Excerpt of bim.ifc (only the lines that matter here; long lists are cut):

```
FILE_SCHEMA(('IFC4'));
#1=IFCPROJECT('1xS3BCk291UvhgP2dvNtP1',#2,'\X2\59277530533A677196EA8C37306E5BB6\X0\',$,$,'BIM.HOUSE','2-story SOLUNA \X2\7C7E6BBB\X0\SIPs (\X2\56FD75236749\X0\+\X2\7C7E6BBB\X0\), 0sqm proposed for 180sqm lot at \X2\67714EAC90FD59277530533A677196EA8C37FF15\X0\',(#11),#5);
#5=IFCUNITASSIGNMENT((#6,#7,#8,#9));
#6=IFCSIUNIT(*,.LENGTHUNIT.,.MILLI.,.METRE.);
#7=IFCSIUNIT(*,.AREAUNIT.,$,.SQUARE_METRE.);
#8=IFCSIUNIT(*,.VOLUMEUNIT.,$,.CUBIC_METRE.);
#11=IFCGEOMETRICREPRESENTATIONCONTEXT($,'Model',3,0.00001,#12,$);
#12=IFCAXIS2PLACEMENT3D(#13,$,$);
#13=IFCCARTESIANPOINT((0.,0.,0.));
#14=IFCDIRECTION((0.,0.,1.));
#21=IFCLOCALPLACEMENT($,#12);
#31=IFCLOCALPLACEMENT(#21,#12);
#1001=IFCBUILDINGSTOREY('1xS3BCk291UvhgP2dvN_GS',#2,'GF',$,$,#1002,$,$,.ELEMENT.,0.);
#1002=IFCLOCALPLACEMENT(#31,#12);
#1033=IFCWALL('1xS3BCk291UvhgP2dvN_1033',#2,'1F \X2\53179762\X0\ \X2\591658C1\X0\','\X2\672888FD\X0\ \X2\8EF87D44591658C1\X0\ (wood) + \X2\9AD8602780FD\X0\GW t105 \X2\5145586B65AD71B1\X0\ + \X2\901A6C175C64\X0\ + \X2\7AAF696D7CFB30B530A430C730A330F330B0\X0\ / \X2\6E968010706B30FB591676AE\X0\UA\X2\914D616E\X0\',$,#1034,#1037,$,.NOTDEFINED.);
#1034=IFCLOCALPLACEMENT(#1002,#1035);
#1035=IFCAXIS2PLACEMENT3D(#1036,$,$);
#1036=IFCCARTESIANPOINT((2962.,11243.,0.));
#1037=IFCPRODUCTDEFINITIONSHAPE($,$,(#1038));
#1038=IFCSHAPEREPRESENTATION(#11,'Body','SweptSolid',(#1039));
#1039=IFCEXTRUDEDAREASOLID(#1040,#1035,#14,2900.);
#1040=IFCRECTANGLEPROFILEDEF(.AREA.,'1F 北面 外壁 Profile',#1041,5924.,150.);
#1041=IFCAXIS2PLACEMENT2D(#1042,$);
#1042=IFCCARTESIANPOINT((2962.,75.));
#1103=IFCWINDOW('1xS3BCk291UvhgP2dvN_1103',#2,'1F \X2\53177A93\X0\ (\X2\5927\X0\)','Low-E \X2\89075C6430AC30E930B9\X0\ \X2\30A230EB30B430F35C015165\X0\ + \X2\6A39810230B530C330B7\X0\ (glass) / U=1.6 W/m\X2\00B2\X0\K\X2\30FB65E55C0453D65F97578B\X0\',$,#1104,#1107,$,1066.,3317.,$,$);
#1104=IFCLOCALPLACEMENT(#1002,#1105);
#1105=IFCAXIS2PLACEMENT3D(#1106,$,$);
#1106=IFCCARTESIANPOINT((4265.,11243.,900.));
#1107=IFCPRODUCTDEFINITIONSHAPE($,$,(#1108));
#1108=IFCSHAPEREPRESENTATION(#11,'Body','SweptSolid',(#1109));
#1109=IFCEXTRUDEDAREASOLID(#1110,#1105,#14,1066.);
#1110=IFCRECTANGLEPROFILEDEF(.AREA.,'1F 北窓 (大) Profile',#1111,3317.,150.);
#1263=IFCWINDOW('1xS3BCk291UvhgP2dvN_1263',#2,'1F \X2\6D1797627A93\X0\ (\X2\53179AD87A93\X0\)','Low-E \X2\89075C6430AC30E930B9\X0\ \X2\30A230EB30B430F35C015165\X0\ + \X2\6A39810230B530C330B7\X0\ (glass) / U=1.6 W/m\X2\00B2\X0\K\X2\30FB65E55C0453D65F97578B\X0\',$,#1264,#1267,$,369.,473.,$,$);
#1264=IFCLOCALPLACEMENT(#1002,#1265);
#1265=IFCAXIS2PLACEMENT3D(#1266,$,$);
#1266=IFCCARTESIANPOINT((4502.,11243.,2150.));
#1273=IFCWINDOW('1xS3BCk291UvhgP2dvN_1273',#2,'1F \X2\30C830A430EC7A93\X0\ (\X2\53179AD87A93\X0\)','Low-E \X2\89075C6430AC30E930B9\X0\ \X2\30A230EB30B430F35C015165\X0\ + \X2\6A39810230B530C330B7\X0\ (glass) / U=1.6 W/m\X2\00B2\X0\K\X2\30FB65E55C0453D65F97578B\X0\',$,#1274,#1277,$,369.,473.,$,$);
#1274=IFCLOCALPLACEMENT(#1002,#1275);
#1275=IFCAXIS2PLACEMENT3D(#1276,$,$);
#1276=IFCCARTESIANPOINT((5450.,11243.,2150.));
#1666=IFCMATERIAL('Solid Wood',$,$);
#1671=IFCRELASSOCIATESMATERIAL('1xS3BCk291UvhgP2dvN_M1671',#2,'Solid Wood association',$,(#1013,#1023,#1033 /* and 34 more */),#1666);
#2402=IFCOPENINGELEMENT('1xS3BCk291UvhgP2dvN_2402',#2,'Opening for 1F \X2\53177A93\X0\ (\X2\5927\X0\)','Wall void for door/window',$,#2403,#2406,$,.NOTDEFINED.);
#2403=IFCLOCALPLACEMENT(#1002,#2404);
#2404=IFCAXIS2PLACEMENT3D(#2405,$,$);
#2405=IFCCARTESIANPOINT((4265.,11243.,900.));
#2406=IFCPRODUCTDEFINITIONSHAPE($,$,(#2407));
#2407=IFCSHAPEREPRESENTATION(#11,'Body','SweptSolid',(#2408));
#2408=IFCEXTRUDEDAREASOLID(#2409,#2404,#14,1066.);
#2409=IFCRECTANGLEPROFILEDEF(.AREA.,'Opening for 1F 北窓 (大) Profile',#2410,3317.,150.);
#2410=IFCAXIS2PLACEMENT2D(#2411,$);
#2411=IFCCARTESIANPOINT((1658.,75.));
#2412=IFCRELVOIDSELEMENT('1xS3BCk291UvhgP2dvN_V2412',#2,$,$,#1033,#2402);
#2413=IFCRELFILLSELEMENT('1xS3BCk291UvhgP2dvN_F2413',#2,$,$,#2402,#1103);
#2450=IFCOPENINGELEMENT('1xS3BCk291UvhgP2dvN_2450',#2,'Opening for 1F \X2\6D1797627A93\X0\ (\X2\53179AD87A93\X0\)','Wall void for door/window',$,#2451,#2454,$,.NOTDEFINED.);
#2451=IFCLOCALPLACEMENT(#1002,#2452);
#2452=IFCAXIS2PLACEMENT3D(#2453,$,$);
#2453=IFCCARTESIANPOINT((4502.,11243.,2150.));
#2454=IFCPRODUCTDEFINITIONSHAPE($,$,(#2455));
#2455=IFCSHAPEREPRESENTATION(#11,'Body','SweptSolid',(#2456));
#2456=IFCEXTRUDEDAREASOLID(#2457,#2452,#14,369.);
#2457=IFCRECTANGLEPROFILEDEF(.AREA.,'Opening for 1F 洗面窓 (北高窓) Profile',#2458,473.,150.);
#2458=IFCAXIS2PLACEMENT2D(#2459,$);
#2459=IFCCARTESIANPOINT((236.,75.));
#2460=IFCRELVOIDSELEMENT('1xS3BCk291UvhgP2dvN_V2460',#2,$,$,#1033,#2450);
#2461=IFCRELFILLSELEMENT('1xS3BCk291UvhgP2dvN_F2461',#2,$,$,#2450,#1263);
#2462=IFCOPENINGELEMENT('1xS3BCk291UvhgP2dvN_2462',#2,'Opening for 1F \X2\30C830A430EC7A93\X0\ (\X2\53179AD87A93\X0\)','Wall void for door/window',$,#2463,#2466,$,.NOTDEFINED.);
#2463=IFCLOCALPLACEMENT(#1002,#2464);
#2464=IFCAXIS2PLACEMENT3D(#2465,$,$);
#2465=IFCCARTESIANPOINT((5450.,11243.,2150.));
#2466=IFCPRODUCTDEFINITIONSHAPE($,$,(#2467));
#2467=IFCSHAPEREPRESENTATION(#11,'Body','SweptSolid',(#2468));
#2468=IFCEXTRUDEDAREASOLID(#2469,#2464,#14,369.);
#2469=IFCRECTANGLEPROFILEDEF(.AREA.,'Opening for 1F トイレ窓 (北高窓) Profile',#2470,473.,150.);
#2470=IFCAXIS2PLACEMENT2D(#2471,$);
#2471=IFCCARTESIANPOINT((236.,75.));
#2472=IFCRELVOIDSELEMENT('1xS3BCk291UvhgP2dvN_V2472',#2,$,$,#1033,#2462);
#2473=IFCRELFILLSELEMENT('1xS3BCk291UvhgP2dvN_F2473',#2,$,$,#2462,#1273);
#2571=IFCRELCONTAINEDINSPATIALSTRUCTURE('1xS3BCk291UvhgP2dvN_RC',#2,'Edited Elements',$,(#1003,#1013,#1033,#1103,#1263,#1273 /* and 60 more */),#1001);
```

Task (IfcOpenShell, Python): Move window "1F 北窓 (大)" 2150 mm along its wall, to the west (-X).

```python
import ifcopenshell
import ifcopenshell.api.geometry
import ifcopenshell.util.placement

model = ifcopenshell.open("bim.ifc")

window = model.by_guid("1xS3BCk291UvhgP2dvN_1103")
opening = window.FillsVoids[0].RelatingOpeningElement
wall = opening.VoidsElements[0].RelatingBuildingElement

wall_matrix = ifcopenshell.util.placement.get_local_placement(wall.ObjectPlacement)
shift = wall_matrix[:3, 0] * -2150.0
before = ifcopenshell.util.placement.get_local_placement(window.ObjectPlacement)[:3, 3].copy()

# The window is not placed relative to its opening, so move both.
for product in (opening, window):
    matrix = ifcopenshell.util.placement.get_local_placement(product.ObjectPlacement)
    matrix[:3, 3] += shift
    ifcopenshell.api.geometry.edit_object_placement(model, product=product, matrix=matrix, is_si=False)

after = ifcopenshell.util.placement.get_local_placement(window.ObjectPlacement)[:3, 3]
print("window moved by", (after - before).round(3) + 0.0)

model.write("bim_edited.ifc")
```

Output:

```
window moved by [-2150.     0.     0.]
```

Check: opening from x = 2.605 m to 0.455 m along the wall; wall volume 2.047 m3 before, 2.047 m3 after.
